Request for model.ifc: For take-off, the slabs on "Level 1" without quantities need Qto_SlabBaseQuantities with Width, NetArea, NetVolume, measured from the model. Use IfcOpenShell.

First a look at what the model holds.

```python
import ifcopenshell
import ifcopenshell.util.element
import ifcopenshell.util.unit

model = ifcopenshell.open("model.ifc")
print(model.schema)
for unit_type in ("LENGTHUNIT", "AREAUNIT", "VOLUMEUNIT"):
    print(unit_type, ifcopenshell.util.unit.calculate_unit_scale(model, unit_type))
storey = next(s for s in model.by_type("IfcBuildingStorey") if s.Name == "Level 1")
slabs = [e for e in ifcopenshell.util.element.get_decomposition(storey) if e.is_a("IfcSlab")]
for e in sorted(slabs, key=lambda e: e.id()):
    print(e.id(), e.is_a(), e.Name, list(ifcopenshell.util.element.get_psets(e, qtos_only=True)), sep=" | ")
```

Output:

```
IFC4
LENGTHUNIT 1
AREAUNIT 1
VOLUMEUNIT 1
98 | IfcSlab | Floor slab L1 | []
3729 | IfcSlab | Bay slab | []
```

```python
import ifcopenshell
import ifcopenshell.api.pset
import ifcopenshell.geom
import ifcopenshell.util.element
import ifcopenshell.util.shape
import ifcopenshell.util.unit

model = ifcopenshell.open("model.ifc")
unit_scale = ifcopenshell.util.unit.calculate_unit_scale(model)
area_scale = ifcopenshell.util.unit.calculate_unit_scale(model, "AREAUNIT")
volume_scale = ifcopenshell.util.unit.calculate_unit_scale(model, "VOLUMEUNIT")
settings = ifcopenshell.geom.settings()

storey = next(s for s in model.by_type("IfcBuildingStorey") if s.Name == "Level 1")
slabs = [e for e in ifcopenshell.util.element.get_decomposition(storey) if e.is_a("IfcSlab")]

for e in sorted(slabs, key=lambda e: e.id()):
    if ifcopenshell.util.element.get_psets(e, qtos_only=True, should_inherit=False):
        continue
    # Geometry comes back in metres, in the element's own axes.
    shape = ifcopenshell.geom.create_shape(settings, e)
    values = {
        "Width": ifcopenshell.util.shape.get_z(shape.geometry) / unit_scale,
        "NetArea": ifcopenshell.util.shape.get_footprint_area(shape.geometry) / area_scale,
        "NetVolume": ifcopenshell.util.shape.get_volume(shape.geometry) / volume_scale,
    }
    qto = ifcopenshell.api.pset.add_qto(model, product=e, name="Qto_SlabBaseQuantities")
    ifcopenshell.api.pset.edit_qto(model, qto=qto, properties=values)
    print(e.id(), {k: round(v, 3) for k, v in values.items()})

model.write("model_updated.ifc")
```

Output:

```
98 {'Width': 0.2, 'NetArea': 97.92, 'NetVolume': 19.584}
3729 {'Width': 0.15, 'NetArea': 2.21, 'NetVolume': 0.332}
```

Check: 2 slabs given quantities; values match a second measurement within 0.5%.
